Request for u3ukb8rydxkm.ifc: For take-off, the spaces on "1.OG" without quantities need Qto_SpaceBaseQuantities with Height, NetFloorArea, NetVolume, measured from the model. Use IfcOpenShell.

First a look at what the model holds.

```python
import ifcopenshell
import ifcopenshell.util.element
import ifcopenshell.util.unit

model = ifcopenshell.open("u3ukb8rydxkm.ifc")
print(model.schema)
for unit_type in ("LENGTHUNIT", "AREAUNIT", "VOLUMEUNIT"):
    print(unit_type, ifcopenshell.util.unit.calculate_unit_scale(model, unit_type))
storey = next(s for s in model.by_type("IfcBuildingStorey") if s.Name == "1.OG")
spaces = [e for e in ifcopenshell.util.element.get_decomposition(storey) if e.is_a("IfcSpace")]
for e in sorted(spaces, key=lambda e: e.id()):
    print(e.id(), e.is_a(), e.Name, list(ifcopenshell.util.element.get_psets(e, qtos_only=True)), sep=" | ")
```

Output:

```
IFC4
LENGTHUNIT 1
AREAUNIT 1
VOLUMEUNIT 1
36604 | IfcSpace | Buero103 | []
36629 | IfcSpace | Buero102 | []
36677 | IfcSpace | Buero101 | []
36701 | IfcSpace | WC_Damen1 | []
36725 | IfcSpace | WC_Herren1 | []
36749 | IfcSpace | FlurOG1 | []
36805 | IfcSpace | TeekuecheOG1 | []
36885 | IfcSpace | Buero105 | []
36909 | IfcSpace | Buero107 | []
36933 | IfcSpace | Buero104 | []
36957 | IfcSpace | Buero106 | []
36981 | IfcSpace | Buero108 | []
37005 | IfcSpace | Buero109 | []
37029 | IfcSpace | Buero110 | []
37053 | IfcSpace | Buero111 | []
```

```python
import ifcopenshell
import ifcopenshell.api.pset
import ifcopenshell.geom
import ifcopenshell.util.element
import ifcopenshell.util.shape
import ifcopenshell.util.unit

model = ifcopenshell.open("u3ukb8rydxkm.ifc")
unit_scale = ifcopenshell.util.unit.calculate_unit_scale(model)
area_scale = ifcopenshell.util.unit.calculate_unit_scale(model, "AREAUNIT")
volume_scale = ifcopenshell.util.unit.calculate_unit_scale(model, "VOLUMEUNIT")
settings = ifcopenshell.geom.settings()

storey = next(s for s in model.by_type("IfcBuildingStorey") if s.Name == "1.OG")
spaces = [e for e in ifcopenshell.util.element.get_decomposition(storey) if e.is_a("IfcSpace")]

for e in sorted(spaces, key=lambda e: e.id()):
    if ifcopenshell.util.element.get_psets(e, qtos_only=True, should_inherit=False):
        continue
    # Geometry comes back in metres, in the element's own axes.
    shape = ifcopenshell.geom.create_shape(settings, e)
    values = {
        "Height": ifcopenshell.util.shape.get_z(shape.geometry) / unit_scale,
        "NetFloorArea": ifcopenshell.util.shape.get_footprint_area(shape.geometry) / area_scale,
        "NetVolume": ifcopenshell.util.shape.get_volume(shape.geometry) / volume_scale,
    }
    qto = ifcopenshell.api.pset.add_qto(model, product=e, name="Qto_SpaceBaseQuantities")
    ifcopenshell.api.pset.edit_qto(model, qto=qto, properties=values)
    print(e.id(), {k: round(v, 3) for k, v in values.items()})

model.write("u3ukb8rydxkm_v2.ifc")
```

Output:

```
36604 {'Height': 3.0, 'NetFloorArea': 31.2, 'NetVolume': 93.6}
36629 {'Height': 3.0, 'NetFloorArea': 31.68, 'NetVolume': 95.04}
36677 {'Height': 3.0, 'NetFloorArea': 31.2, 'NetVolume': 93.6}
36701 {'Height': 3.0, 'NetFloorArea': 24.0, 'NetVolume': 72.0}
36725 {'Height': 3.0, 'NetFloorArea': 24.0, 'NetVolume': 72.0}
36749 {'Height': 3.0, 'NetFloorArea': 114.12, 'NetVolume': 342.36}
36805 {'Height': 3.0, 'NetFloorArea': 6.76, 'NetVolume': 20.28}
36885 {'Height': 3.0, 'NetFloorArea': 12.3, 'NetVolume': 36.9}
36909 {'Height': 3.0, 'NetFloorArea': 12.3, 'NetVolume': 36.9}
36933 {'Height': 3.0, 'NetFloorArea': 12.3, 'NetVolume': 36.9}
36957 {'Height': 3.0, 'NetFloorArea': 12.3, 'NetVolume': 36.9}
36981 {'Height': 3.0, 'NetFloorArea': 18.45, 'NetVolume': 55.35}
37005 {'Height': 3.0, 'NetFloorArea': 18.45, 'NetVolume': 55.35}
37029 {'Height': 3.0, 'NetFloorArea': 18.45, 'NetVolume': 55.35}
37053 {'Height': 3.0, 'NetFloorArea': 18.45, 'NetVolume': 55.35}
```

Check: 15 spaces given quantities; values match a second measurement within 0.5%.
